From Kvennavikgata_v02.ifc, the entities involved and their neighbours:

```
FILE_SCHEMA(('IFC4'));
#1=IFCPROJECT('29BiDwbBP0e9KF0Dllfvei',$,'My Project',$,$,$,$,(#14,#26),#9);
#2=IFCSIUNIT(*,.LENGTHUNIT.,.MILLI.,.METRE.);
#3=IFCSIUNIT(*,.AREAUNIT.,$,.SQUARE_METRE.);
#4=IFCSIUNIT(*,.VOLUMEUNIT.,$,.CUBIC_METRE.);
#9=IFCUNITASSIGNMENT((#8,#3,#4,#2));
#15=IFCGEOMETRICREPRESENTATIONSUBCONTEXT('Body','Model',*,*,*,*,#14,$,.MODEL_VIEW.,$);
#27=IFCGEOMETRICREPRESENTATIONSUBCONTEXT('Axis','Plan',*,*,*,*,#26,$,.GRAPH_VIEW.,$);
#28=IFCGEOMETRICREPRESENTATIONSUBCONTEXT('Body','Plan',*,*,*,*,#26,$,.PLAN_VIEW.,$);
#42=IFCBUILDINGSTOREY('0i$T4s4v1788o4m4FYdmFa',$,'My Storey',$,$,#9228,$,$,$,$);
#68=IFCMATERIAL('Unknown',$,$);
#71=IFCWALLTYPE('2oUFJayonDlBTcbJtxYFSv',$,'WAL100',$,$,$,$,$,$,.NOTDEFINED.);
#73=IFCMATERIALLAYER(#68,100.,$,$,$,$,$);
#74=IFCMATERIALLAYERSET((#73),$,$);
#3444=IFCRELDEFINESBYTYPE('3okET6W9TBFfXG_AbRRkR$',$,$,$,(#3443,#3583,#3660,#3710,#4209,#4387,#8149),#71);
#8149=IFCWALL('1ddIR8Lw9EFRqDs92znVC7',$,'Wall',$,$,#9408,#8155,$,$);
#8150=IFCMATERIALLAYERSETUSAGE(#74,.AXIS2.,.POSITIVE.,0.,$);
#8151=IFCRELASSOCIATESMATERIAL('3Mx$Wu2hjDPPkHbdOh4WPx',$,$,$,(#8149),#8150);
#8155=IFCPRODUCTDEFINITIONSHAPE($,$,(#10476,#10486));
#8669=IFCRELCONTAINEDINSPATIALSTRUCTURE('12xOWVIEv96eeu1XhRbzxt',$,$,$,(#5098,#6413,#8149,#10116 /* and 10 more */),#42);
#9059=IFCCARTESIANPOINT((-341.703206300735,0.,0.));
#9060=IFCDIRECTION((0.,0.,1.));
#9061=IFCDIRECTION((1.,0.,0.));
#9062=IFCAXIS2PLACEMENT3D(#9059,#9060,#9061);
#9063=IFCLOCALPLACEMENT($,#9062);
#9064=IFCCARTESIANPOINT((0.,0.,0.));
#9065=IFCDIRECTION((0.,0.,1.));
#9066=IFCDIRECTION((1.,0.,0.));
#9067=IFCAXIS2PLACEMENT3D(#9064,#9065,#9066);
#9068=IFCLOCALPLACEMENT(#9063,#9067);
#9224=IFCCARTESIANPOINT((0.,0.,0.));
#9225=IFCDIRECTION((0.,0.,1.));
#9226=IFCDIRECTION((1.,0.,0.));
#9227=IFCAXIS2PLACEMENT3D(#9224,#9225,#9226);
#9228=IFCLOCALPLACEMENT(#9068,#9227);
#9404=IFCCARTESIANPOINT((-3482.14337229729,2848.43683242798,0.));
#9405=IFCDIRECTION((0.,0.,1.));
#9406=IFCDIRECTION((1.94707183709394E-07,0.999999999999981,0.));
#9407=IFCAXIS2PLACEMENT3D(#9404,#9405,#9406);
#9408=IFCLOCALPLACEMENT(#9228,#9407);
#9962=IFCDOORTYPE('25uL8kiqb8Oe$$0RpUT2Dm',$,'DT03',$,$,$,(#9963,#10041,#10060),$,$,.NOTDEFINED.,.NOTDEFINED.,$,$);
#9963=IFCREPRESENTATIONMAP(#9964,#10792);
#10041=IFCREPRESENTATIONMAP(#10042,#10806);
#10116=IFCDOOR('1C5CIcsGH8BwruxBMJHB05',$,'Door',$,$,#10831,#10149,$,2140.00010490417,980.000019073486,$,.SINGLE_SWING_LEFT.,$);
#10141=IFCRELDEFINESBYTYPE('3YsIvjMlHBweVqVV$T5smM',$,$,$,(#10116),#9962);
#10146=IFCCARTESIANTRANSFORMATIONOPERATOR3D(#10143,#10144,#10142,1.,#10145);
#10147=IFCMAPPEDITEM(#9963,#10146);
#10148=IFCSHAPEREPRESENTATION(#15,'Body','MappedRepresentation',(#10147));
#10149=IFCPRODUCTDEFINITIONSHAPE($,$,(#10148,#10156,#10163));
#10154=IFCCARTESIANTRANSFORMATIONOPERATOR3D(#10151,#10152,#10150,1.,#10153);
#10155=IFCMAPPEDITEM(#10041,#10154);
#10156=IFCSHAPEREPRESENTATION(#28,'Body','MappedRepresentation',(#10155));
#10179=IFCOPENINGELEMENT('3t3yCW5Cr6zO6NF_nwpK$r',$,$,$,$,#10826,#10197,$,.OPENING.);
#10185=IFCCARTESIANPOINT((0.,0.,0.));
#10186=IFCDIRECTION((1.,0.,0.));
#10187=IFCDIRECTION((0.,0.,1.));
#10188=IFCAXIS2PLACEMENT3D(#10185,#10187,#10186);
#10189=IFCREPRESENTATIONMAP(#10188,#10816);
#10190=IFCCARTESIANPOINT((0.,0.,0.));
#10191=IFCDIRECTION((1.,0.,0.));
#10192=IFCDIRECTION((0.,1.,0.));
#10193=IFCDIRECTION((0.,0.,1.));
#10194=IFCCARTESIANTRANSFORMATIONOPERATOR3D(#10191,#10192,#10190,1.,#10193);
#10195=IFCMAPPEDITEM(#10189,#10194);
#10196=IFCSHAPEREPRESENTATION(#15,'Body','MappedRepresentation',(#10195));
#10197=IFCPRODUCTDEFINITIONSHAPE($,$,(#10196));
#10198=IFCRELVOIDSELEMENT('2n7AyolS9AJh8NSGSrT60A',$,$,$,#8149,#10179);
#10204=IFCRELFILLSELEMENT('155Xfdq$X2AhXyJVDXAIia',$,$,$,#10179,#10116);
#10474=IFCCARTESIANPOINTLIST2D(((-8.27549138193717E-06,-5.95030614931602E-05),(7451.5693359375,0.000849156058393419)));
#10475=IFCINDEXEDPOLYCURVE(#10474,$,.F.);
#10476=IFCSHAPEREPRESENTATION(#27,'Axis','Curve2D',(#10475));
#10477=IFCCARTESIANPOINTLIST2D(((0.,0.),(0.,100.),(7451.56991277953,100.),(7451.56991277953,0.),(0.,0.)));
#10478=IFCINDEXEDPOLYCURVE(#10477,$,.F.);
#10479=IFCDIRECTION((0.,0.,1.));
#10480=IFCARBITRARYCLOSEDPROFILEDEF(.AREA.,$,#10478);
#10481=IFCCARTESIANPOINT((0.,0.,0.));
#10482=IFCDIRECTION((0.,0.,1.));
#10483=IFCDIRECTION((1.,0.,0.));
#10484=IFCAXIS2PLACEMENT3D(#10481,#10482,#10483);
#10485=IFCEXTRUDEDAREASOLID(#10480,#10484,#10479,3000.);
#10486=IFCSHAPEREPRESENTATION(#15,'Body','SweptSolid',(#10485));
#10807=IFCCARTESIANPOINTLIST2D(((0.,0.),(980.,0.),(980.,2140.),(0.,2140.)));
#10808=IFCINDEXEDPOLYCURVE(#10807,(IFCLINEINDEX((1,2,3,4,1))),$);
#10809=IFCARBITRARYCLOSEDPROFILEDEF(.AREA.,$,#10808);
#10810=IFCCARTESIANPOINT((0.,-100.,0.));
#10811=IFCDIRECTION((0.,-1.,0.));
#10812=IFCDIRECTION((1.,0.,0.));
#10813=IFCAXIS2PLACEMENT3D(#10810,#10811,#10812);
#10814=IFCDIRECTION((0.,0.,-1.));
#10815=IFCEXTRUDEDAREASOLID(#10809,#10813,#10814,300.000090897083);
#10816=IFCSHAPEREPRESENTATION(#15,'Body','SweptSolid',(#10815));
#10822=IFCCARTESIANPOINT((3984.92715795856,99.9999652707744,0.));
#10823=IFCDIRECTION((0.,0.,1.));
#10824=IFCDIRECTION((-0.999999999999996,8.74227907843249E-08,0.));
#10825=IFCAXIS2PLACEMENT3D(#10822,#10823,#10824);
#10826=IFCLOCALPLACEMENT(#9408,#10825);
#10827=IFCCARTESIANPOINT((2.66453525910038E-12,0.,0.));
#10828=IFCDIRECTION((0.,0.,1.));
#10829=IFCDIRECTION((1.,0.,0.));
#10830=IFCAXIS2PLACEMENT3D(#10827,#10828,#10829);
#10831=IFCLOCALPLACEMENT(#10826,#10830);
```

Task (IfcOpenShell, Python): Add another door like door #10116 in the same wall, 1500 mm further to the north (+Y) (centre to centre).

```python
import ifcopenshell
import ifcopenshell.api.feature
import ifcopenshell.api.geometry
import ifcopenshell.api.root
import ifcopenshell.geom
import ifcopenshell.util.element
import ifcopenshell.util.placement
import ifcopenshell.util.shape
import ifcopenshell.util.unit

model = ifcopenshell.open("Kvennavikgata_v02.ifc")
unit_scale = ifcopenshell.util.unit.calculate_unit_scale(model)
settings = ifcopenshell.geom.settings()


def volume(element):
    """Net volume in cubic metres, openings subtracted."""
    shape = ifcopenshell.geom.create_shape(settings, element)
    return ifcopenshell.util.shape.get_volume(shape.geometry)


door = model.by_guid("1C5CIcsGH8BwruxBMJHB05")
opening = door.FillsVoids[0].RelatingOpeningElement
wall = opening.VoidsElements[0].RelatingBuildingElement
before = volume(wall)
shift = ifcopenshell.util.placement.get_local_placement(wall.ObjectPlacement)[:3, 0] * 1.5 / unit_scale

# copy_class copies the void relationship, type, container and properties, but no geometry.
new_opening = ifcopenshell.api.root.copy_class(model, product=opening)
new_opening.Representation = ifcopenshell.util.element.copy_deep(
    model, opening.Representation, exclude=["IfcGeometricRepresentationContext", "IfcRepresentationMap"]
)
new_door = ifcopenshell.api.root.copy_class(model, product=door)
new_door.Representation = ifcopenshell.util.element.copy_deep(
    model, door.Representation, exclude=["IfcGeometricRepresentationContext", "IfcRepresentationMap"]
)
ifcopenshell.api.feature.add_filling(model, opening=new_opening, element=new_door)

for old, new in ((opening, new_opening), (door, new_door)):
    matrix = ifcopenshell.util.placement.get_local_placement(old.ObjectPlacement)
    matrix[:3, 3] += shift
    ifcopenshell.api.geometry.edit_object_placement(model, product=new, matrix=matrix, is_si=False)

after = volume(wall)

print(f"wall volume {before:.3f} -> {after:.3f} m3")

model.write("Kvennavikgata_v02_v2.ifc")
```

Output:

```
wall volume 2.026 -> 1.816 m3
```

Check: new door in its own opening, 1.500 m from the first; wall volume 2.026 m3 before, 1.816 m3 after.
